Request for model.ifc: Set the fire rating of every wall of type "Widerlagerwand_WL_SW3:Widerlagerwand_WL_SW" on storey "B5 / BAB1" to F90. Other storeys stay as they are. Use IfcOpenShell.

First a look at what the model holds.

```python
import ifcopenshell
import ifcopenshell.util.element

model = ifcopenshell.open("model.ifc")
print(model.schema)
storey = next(s for s in model.by_type("IfcBuildingStorey") if s.Name == "B5 / BAB1")
walls = [e for e in ifcopenshell.util.element.get_decomposition(storey) if e.is_a("IfcWall")]
seen = {}
for e in walls:
    element_type = ifcopenshell.util.element.get_type(e)
    key = (element_type.Name if element_type != e and element_type else None, ifcopenshell.util.element.get_pset(e, "Pset_WallCommon", "FireRating"))
    seen[key] = seen.get(key, 0) + 1
for (name, value), count in sorted(seen.items(), key=str):
    print(count, "x", name, "|", value)
```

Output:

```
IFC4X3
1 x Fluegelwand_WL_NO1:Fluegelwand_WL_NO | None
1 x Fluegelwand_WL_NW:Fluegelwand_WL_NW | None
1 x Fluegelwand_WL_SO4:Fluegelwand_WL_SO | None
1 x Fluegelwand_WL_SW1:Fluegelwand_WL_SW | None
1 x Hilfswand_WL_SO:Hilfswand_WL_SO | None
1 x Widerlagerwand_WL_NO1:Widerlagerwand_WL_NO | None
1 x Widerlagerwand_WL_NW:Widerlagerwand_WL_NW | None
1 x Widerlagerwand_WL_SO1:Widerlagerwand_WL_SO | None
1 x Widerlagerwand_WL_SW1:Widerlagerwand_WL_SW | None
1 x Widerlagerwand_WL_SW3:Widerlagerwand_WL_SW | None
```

```python
import ifcopenshell
import ifcopenshell.api.pset
import ifcopenshell.util.element

model = ifcopenshell.open("model.ifc")

storey = next(s for s in model.by_type("IfcBuildingStorey") if s.Name == "B5 / BAB1")
walls = [e for e in ifcopenshell.util.element.get_decomposition(storey) if e.is_a("IfcWall")]

count = 0
for e in walls:
    element_type = ifcopenshell.util.element.get_type(e)
    if element_type in (None, e) or element_type.Name != "Widerlagerwand_WL_SW3:Widerlagerwand_WL_SW":
        continue
    # add_pset returns the element's existing set when there is one.
    pset = ifcopenshell.api.pset.add_pset(model, product=e, name="Pset_WallCommon")
    ifcopenshell.api.pset.edit_pset(model, pset=pset, properties={"FireRating": "F90"})
    count += 1

print(count, "walls updated")

model.write("model_updated.ifc")
```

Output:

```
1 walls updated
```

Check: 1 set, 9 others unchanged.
